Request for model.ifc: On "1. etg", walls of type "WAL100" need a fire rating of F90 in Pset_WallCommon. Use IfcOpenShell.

First a look at what the model holds.

```python
import ifcopenshell
import ifcopenshell.util.element

model = ifcopenshell.open("model.ifc")
print(model.schema)
storey = next(s for s in model.by_type("IfcBuildingStorey") if s.Name == "1. etg")
walls = [e for e in ifcopenshell.util.element.get_decomposition(storey) if e.is_a("IfcWall")]
seen = {}
for e in walls:
    element_type = ifcopenshell.util.element.get_type(e)
    key = (element_type.Name if element_type != e and element_type else None, ifcopenshell.util.element.get_pset(e, "Pset_WallCommon", "FireRating"))
    seen[key] = seen.get(key, 0) + 1
for (name, value), count in sorted(seen.items(), key=str):
    print(count, "x", name, "|", value)
```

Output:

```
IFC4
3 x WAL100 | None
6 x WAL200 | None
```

```python
import ifcopenshell
import ifcopenshell.api.pset
import ifcopenshell.util.element

model = ifcopenshell.open("model.ifc")

storey = next(s for s in model.by_type("IfcBuildingStorey") if s.Name == "1. etg")
walls = [e for e in ifcopenshell.util.element.get_decomposition(storey) if e.is_a("IfcWall")]

count = 0
for e in walls:
    element_type = ifcopenshell.util.element.get_type(e)
    if element_type in (None, e) or element_type.Name != "WAL100":
        continue
    # add_pset returns the element's existing set when there is one.
    pset = ifcopenshell.api.pset.add_pset(model, product=e, name="Pset_WallCommon")
    ifcopenshell.api.pset.edit_pset(model, pset=pset, properties={"FireRating": "F90"})
    count += 1

print(count, "walls updated")

model.write("model_v2.ifc")
```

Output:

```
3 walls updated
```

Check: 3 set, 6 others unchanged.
